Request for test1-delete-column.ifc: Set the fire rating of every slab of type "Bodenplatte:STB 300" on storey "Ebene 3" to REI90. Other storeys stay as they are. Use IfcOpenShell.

First a look at what the model holds.

```python
import ifcopenshell
import ifcopenshell.util.element

model = ifcopenshell.open("test1-delete-column.ifc")
print(model.schema)
storey = next(s for s in model.by_type("IfcBuildingStorey") if s.Name == "Ebene 3")
slabs = [e for e in ifcopenshell.util.element.get_decomposition(storey) if e.is_a("IfcSlab")]
seen = {}
for e in slabs:
    element_type = ifcopenshell.util.element.get_type(e)
    key = (element_type.Name if element_type != e and element_type else None, ifcopenshell.util.element.get_pset(e, "Pset_SlabCommon", "FireRating"))
    seen[key] = seen.get(key, 0) + 1
for (name, value), count in sorted(seen.items(), key=str):
    print(count, "x", name, "|", value)
```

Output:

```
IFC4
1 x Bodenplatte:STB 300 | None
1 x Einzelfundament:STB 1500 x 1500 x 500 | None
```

```python
import ifcopenshell
import ifcopenshell.api.pset
import ifcopenshell.util.element

model = ifcopenshell.open("test1-delete-column.ifc")

storey = next(s for s in model.by_type("IfcBuildingStorey") if s.Name == "Ebene 3")
slabs = [e for e in ifcopenshell.util.element.get_decomposition(storey) if e.is_a("IfcSlab")]

count = 0
for e in slabs:
    element_type = ifcopenshell.util.element.get_type(e)
    if element_type in (None, e) or element_type.Name != "Bodenplatte:STB 300":
        continue
    # add_pset returns the element's existing set when there is one.
    pset = ifcopenshell.api.pset.add_pset(model, product=e, name="Pset_SlabCommon")
    ifcopenshell.api.pset.edit_pset(model, pset=pset, properties={"FireRating": "REI90"})
    count += 1

print(count, "slabs updated")

model.write("test1-delete-column_rev.ifc")
```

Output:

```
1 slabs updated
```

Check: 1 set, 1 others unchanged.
